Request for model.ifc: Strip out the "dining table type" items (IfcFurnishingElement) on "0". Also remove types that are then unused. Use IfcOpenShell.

First a look at what the model holds.

```python
import ifcopenshell
import ifcopenshell.util.element

model = ifcopenshell.open("model.ifc")
print(model.schema)
storey = next(s for s in model.by_type("IfcBuildingStorey") if s.Name == "0")
furniture = [e for e in ifcopenshell.util.element.get_decomposition(storey) if e.is_a("IfcFurnishingElement")]
seen = {}
for e in furniture:
    element_type = ifcopenshell.util.element.get_type(e)
    name = element_type.Name if element_type not in (None, e) else None
    seen[name] = seen.get(name, 0) + 1
for name, count in sorted(seen.items(), key=str):
    print(count, "x", name)
```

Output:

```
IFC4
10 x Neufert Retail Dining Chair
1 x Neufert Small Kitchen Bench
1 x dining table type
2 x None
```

```python
import ifcopenshell
import ifcopenshell.api.root
import ifcopenshell.util.element

model = ifcopenshell.open("model.ifc")

storey = next(s for s in model.by_type("IfcBuildingStorey") if s.Name == "0")
furniture = [e for e in ifcopenshell.util.element.get_decomposition(storey) if e.is_a("IfcFurnishingElement")]
targets = [e for e in furniture if (t := ifcopenshell.util.element.get_type(e)) not in (None, e) and t.Name == "dining table type"]
types = {ifcopenshell.util.element.get_type(e) for e in targets} - {None, *targets}

for e in targets:
    ifcopenshell.api.root.remove_product(model, product=e)
print(len(targets), "removed")

unused = [t for t in types if not ifcopenshell.util.element.get_types(t)]
for t in unused:
    ifcopenshell.api.root.remove_product(model, product=t)
print(len(unused), "unused types removed")

model.write("model_v2.ifc")
```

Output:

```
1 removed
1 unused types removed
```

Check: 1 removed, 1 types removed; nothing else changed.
